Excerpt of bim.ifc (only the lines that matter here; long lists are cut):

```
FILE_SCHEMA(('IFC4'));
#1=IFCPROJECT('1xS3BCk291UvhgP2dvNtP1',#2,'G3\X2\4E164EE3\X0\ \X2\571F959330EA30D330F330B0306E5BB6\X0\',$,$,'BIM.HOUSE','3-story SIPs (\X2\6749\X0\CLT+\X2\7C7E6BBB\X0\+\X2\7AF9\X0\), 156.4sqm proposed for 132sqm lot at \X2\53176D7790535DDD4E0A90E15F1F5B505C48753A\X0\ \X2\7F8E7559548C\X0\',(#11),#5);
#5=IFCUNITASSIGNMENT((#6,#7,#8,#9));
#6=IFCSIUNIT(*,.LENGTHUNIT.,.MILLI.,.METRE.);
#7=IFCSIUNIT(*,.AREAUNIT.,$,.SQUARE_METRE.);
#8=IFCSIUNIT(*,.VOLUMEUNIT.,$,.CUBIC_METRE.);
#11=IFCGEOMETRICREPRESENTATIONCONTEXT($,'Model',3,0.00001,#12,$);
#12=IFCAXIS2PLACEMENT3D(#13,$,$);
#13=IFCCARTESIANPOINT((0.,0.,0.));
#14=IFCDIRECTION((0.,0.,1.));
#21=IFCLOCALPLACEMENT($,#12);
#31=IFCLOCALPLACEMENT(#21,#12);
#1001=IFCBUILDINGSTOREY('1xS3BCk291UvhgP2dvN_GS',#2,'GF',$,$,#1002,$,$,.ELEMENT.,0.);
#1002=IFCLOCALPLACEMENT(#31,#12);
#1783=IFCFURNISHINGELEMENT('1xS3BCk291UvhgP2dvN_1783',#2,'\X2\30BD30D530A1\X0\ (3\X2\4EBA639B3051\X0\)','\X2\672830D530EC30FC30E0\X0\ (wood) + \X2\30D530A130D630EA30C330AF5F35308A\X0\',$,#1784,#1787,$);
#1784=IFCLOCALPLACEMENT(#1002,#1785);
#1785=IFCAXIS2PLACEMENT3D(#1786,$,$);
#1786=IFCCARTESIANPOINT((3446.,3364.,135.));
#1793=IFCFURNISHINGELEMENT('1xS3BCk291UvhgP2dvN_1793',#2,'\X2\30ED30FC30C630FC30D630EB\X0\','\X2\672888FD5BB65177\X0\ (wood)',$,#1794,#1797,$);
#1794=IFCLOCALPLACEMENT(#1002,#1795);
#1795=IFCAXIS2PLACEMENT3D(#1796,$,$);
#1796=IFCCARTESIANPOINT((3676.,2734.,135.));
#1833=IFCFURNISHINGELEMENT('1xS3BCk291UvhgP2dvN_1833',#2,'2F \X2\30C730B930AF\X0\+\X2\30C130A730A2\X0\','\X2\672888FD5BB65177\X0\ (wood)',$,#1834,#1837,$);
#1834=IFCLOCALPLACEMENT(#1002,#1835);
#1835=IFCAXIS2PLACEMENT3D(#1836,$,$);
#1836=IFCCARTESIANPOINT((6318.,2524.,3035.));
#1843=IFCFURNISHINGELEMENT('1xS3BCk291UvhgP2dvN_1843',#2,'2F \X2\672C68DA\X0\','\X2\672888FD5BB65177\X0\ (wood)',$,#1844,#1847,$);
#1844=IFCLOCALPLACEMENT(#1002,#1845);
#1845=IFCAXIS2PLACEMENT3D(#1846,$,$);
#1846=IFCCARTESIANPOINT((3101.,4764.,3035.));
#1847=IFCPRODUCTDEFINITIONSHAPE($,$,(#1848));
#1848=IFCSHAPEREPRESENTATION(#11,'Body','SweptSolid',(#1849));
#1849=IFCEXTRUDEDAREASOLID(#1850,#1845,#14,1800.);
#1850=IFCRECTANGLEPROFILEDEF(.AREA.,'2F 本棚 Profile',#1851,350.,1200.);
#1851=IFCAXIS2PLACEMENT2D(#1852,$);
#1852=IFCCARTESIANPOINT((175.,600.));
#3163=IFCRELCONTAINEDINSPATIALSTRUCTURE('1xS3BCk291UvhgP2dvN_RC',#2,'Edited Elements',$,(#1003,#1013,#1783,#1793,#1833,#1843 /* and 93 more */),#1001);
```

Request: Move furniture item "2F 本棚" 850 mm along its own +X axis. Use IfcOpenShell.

```python
import ifcopenshell
import ifcopenshell.api.geometry
import ifcopenshell.util.placement
import ifcopenshell.util.unit

model = ifcopenshell.open("bim.ifc")
unit_scale = ifcopenshell.util.unit.calculate_unit_scale(model)

item = model.by_guid("1xS3BCk291UvhgP2dvN_1843")
matrix = ifcopenshell.util.placement.get_local_placement(item.ObjectPlacement)
matrix[:3, 3] += matrix[:3, 0] * 0.85 / unit_scale
ifcopenshell.api.geometry.edit_object_placement(model, product=item, matrix=matrix, is_si=False)

print(ifcopenshell.util.placement.get_local_placement(item.ObjectPlacement).round(3) + 0.0)

model.write("bim_updated.ifc")
```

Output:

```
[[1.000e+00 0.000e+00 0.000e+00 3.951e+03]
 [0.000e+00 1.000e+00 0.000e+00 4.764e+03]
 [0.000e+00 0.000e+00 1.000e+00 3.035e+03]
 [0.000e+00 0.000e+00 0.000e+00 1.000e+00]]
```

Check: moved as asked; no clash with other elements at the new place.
